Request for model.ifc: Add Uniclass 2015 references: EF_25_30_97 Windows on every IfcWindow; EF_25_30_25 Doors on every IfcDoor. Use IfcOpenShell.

First a look at what the model holds.

```python
import ifcopenshell

model = ifcopenshell.open("model.ifc")
print(model.schema)
print("classifications:", [c.Name for c in model.by_type("IfcClassification")])
for ifc_class in ("IfcDoor", "IfcRoof", "IfcStair", "IfcWall", "IfcWindow"):
    print(ifc_class, len(model.by_type(ifc_class)))
```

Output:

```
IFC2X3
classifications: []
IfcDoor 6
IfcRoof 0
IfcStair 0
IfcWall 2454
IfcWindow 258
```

```python
import ifcopenshell
import ifcopenshell.api.classification

model = ifcopenshell.open("model.ifc")

# IFC2X3 requires Source and Edition and has no link from the project to the system.
system = model.create_entity("IfcClassification", Source="NBS", Edition="2015", Name="Uniclass 2015")

codes = {
    "IfcWindow": ("EF_25_30_97", "Windows"),
    "IfcDoor": ("EF_25_30_25", "Doors"),
}
for ifc_class, (code, name) in codes.items():
    products = model.by_type(ifc_class)
    ifcopenshell.api.classification.add_reference(
        model, products=products, classification=system, identification=code, name=name
    )
    print(code, len(products))

model.write("model_rev.ifc")
```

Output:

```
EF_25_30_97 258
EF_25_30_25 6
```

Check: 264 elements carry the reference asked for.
